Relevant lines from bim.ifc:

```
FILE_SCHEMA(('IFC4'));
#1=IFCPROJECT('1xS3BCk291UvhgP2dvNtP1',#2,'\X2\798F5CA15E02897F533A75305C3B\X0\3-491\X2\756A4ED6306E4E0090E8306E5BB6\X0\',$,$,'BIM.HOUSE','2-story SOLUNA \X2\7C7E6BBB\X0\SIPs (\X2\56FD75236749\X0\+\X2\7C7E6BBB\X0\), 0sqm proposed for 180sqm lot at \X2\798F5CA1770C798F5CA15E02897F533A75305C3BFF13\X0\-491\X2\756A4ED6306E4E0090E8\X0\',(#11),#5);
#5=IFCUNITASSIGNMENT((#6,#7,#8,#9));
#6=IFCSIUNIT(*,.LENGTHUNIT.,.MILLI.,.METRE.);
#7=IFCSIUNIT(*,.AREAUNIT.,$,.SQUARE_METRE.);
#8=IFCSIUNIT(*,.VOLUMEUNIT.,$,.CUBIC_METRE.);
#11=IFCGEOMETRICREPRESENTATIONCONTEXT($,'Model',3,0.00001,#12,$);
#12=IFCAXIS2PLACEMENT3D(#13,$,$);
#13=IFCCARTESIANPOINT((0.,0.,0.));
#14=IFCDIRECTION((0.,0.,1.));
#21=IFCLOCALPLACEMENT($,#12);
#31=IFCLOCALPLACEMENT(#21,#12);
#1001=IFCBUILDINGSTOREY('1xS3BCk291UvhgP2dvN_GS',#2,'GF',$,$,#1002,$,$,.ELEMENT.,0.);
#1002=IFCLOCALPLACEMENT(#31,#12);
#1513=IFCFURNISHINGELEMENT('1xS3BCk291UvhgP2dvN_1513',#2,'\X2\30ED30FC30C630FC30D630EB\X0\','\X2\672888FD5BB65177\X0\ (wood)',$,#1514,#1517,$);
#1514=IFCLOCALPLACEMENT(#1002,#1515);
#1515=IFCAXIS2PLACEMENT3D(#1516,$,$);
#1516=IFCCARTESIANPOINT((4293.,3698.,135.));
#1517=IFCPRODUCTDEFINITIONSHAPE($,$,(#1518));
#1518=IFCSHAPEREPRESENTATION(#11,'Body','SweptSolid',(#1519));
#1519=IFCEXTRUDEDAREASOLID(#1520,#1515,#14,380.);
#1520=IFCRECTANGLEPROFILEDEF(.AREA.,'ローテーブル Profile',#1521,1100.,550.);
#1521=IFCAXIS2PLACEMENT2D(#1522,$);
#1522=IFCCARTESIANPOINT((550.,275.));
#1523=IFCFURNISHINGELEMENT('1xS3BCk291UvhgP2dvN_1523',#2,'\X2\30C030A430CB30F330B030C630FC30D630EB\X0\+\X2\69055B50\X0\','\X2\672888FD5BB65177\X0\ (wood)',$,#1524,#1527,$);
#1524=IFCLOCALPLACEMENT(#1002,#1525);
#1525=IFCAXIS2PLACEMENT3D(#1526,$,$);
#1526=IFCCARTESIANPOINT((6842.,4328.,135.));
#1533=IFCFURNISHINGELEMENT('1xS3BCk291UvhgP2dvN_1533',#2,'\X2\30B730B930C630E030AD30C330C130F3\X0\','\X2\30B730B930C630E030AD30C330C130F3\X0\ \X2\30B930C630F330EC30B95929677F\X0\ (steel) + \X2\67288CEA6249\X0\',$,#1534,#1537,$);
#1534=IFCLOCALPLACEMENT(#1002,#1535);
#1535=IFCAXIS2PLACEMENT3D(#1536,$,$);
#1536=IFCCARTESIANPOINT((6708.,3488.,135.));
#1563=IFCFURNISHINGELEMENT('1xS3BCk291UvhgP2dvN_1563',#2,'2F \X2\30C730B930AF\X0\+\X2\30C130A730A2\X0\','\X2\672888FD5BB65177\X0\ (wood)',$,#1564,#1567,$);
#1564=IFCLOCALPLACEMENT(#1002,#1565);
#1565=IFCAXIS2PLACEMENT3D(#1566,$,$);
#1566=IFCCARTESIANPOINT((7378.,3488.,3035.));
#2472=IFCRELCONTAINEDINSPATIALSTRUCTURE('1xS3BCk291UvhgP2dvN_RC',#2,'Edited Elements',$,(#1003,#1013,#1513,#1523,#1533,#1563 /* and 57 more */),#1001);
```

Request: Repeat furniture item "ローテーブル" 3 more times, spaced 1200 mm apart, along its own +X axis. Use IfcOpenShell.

```python
import ifcopenshell
import ifcopenshell.api.geometry
import ifcopenshell.api.root
import ifcopenshell.util.element
import ifcopenshell.util.placement

model = ifcopenshell.open("bim.ifc")


def reuse_history(source, copy):
    """copy_class also copies each property set's owner history, people and application; keep the originals."""
    for rel in copy.IsDefinedBy:
        if rel.is_a("IfcRelDefinesByProperties") and (history := rel.RelatingPropertyDefinition.OwnerHistory):
            rel.RelatingPropertyDefinition.OwnerHistory = source.OwnerHistory
            ifcopenshell.util.element.remove_deep2(model, history)


source = model.by_guid("1xS3BCk291UvhgP2dvN_1513")
base = ifcopenshell.util.placement.get_local_placement(source.ObjectPlacement)
step = base[:3, 0] * 1200.0

for i in range(1, 4):
    copy = ifcopenshell.api.root.copy_class(model, product=source)
    copy.Representation = ifcopenshell.util.element.copy_deep(
        model, source.Representation, exclude=["IfcGeometricRepresentationContext", "IfcRepresentationMap"]
    )
    reuse_history(source, copy)
    matrix = base.copy()
    matrix[:3, 3] += i * step
    print("added at", matrix[:3, 3].round(3) + 0.0)
    ifcopenshell.api.geometry.edit_object_placement(model, product=copy, matrix=matrix, is_si=False)

model.write("bim_updated.ifc")
```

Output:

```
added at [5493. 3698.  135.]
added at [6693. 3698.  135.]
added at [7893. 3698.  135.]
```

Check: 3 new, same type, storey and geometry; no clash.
